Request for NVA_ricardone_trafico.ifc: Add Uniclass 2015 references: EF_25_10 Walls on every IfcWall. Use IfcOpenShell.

First a look at what the model holds.

```python
import ifcopenshell

model = ifcopenshell.open("NVA_ricardone_trafico.ifc")
print(model.schema)
print("classifications:", [c.Name for c in model.by_type("IfcClassification")])
for ifc_class in ("IfcDoor", "IfcRoof", "IfcStair", "IfcWall", "IfcWindow"):
    print(ifc_class, len(model.by_type(ifc_class)))
```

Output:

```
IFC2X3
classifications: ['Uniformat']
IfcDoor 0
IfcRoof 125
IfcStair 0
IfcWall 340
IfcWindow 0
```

```python
import ifcopenshell
import ifcopenshell.api.classification

model = ifcopenshell.open("NVA_ricardone_trafico.ifc")

# IFC2X3 requires Source and Edition and has no link from the project to the system.
system = model.create_entity("IfcClassification", Source="NBS", Edition="2015", Name="Uniclass 2015")

codes = {
    "IfcWall": ("EF_25_10", "Walls"),
}
for ifc_class, (code, name) in codes.items():
    products = model.by_type(ifc_class)
    ifcopenshell.api.classification.add_reference(
        model, products=products, classification=system, identification=code, name=name
    )
    print(code, len(products))

model.write("NVA_ricardone_trafico_rev.ifc")
```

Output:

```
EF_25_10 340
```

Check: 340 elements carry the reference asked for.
